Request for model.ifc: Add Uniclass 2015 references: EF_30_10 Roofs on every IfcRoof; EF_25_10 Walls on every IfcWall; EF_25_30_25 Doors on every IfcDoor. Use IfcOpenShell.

First a look at what the model holds.

```python
import ifcopenshell

model = ifcopenshell.open("model.ifc")
print(model.schema)
print("classifications:", [c.Name for c in model.by_type("IfcClassification")])
for ifc_class in ("IfcDoor", "IfcRoof", "IfcStair", "IfcWall", "IfcWindow"):
    print(ifc_class, len(model.by_type(ifc_class)))
```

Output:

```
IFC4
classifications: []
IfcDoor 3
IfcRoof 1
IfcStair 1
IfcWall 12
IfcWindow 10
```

```python
import ifcopenshell
import ifcopenshell.api.classification

model = ifcopenshell.open("model.ifc")

system = ifcopenshell.api.classification.add_classification(model, classification="Uniclass 2015")

codes = {
    "IfcRoof": ("EF_30_10", "Roofs"),
    "IfcWall": ("EF_25_10", "Walls"),
    "IfcDoor": ("EF_25_30_25", "Doors"),
}
for ifc_class, (code, name) in codes.items():
    products = model.by_type(ifc_class)
    ifcopenshell.api.classification.add_reference(
        model, products=products, classification=system, identification=code, name=name
    )
    print(code, len(products))

model.write("model_edited.ifc")
```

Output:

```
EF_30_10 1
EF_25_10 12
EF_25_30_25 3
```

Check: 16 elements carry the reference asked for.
